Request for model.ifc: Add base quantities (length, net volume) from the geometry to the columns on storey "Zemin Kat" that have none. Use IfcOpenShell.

First a look at what the model holds.

```python
import ifcopenshell
import ifcopenshell.util.element
import ifcopenshell.util.unit

model = ifcopenshell.open("model.ifc")
print(model.schema)
for unit_type in ("LENGTHUNIT", "AREAUNIT", "VOLUMEUNIT"):
    print(unit_type, ifcopenshell.util.unit.calculate_unit_scale(model, unit_type))
storey = next(s for s in model.by_type("IfcBuildingStorey") if s.Name == "Zemin Kat")
columns = [e for e in ifcopenshell.util.element.get_decomposition(storey) if e.is_a("IfcColumn")]
for e in sorted(columns, key=lambda e: e.id()):
    print(e.id(), e.is_a(), e.Name, list(ifcopenshell.util.element.get_psets(e, qtos_only=True)), sep=" | ")
```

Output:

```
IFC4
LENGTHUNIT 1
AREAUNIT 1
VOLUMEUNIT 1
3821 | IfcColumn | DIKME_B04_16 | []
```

```python
import ifcopenshell
import ifcopenshell.api.pset
import ifcopenshell.geom
import ifcopenshell.util.element
import ifcopenshell.util.shape
import ifcopenshell.util.unit

model = ifcopenshell.open("model.ifc")
unit_scale = ifcopenshell.util.unit.calculate_unit_scale(model)
volume_scale = ifcopenshell.util.unit.calculate_unit_scale(model, "VOLUMEUNIT")
settings = ifcopenshell.geom.settings()

storey = next(s for s in model.by_type("IfcBuildingStorey") if s.Name == "Zemin Kat")
columns = [e for e in ifcopenshell.util.element.get_decomposition(storey) if e.is_a("IfcColumn")]

for e in sorted(columns, key=lambda e: e.id()):
    if ifcopenshell.util.element.get_psets(e, qtos_only=True, should_inherit=False):
        continue
    # Geometry comes back in metres, in the element's own axes.
    shape = ifcopenshell.geom.create_shape(settings, e)
    values = {
        "Length": ifcopenshell.util.shape.get_z(shape.geometry) / unit_scale,
        "NetVolume": ifcopenshell.util.shape.get_volume(shape.geometry) / volume_scale,
    }
    qto = ifcopenshell.api.pset.add_qto(model, product=e, name="Qto_ColumnBaseQuantities")
    ifcopenshell.api.pset.edit_qto(model, qto=qto, properties=values)
    print(e.id(), {k: round(v, 3) for k, v in values.items()})

model.write("model_updated.ifc")
```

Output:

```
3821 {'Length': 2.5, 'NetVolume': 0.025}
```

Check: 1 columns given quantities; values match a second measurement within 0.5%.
